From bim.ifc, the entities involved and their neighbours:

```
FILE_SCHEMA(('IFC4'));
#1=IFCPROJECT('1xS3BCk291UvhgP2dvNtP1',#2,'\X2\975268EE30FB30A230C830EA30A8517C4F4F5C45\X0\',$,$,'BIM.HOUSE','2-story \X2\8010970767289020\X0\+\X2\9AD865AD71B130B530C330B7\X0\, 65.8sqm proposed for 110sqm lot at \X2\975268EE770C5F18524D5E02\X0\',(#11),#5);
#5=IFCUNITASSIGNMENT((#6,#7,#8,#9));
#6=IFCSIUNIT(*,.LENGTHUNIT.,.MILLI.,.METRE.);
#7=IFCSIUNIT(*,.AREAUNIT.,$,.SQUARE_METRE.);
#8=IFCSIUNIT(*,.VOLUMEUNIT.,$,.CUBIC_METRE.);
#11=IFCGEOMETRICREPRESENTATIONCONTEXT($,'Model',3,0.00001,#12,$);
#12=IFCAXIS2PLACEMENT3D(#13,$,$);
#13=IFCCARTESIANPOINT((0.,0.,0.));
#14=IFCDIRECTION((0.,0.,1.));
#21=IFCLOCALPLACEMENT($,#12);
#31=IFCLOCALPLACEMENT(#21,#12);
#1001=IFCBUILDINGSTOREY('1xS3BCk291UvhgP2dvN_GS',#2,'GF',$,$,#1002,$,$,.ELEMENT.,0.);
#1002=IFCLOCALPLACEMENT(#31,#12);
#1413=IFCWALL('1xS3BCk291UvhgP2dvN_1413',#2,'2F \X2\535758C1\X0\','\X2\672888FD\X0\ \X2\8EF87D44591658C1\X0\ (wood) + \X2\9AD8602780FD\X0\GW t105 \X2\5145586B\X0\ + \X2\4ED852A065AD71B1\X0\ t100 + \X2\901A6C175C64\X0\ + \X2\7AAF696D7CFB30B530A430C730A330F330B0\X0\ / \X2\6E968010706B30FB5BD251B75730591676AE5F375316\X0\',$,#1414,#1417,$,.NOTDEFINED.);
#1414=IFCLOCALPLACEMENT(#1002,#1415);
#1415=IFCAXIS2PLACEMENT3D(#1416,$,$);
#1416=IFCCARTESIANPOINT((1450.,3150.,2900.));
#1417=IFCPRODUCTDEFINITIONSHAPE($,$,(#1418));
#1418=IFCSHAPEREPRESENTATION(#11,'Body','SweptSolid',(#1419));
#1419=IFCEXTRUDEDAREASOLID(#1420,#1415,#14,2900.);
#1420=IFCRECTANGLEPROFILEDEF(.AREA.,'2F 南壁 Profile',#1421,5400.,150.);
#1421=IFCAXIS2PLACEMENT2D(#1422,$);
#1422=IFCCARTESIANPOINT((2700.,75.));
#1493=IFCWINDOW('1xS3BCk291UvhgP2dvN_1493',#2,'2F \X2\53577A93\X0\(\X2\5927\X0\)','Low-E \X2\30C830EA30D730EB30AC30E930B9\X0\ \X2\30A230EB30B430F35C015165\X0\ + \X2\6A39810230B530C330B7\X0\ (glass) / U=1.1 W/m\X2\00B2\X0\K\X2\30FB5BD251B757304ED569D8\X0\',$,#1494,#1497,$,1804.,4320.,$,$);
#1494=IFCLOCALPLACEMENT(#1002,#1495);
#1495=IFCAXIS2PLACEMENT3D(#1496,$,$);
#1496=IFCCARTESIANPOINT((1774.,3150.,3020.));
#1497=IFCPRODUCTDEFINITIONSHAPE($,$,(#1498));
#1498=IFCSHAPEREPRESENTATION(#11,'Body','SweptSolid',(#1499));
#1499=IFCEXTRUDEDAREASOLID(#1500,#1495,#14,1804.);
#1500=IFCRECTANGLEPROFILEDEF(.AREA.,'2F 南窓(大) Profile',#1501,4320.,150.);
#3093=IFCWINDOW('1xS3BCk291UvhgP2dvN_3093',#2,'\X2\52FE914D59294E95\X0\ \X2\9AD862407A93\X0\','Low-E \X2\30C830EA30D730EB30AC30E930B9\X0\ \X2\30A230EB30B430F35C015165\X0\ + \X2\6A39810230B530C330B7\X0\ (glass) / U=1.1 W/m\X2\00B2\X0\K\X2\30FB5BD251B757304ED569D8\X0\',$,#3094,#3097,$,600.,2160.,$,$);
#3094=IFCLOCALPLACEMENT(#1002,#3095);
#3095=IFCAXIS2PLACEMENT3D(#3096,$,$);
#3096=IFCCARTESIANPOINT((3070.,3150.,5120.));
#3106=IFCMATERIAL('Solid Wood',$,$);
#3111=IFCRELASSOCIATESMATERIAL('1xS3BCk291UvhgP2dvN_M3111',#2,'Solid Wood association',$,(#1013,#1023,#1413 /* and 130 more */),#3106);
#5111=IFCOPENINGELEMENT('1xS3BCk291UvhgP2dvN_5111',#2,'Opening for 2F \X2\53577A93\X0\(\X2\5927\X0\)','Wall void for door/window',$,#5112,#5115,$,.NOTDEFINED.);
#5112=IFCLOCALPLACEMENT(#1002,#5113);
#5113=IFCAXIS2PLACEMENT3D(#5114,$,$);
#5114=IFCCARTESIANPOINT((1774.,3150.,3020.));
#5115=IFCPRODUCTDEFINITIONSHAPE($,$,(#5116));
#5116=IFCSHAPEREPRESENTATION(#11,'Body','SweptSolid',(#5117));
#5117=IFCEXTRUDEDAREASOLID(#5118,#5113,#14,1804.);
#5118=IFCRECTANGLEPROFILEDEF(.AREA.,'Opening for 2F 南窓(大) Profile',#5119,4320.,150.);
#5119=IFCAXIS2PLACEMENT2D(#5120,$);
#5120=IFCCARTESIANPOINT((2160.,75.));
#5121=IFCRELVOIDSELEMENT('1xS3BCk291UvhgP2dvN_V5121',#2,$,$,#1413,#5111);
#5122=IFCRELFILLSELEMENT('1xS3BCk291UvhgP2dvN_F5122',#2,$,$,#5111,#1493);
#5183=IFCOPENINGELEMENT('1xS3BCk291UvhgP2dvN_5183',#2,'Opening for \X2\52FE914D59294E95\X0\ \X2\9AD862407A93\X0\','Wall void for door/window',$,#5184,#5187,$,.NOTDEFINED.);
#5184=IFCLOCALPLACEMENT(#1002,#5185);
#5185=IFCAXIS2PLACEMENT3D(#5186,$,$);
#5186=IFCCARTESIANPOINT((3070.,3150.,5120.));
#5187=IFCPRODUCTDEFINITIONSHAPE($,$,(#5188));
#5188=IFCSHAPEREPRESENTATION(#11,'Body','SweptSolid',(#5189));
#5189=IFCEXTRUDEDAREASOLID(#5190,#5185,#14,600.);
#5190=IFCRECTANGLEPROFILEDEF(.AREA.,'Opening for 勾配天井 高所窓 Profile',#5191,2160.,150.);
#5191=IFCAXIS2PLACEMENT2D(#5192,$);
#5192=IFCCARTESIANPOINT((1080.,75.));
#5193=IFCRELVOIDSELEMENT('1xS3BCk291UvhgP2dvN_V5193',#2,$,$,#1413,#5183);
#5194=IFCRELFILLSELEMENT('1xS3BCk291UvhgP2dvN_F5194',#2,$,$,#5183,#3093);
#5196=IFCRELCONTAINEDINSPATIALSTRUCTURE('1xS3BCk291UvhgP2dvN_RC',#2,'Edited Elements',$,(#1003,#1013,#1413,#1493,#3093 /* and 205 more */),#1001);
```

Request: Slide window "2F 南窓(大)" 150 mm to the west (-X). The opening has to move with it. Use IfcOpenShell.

```python
import ifcopenshell
import ifcopenshell.api.geometry
import ifcopenshell.util.placement

model = ifcopenshell.open("bim.ifc")

window = model.by_id(1493)
opening = window.FillsVoids[0].RelatingOpeningElement
wall = opening.VoidsElements[0].RelatingBuildingElement

wall_matrix = ifcopenshell.util.placement.get_local_placement(wall.ObjectPlacement)
shift = wall_matrix[:3, 0] * -150.0
before = ifcopenshell.util.placement.get_local_placement(window.ObjectPlacement)[:3, 3].copy()

# The window is not placed relative to its opening, so move both.
for product in (opening, window):
    matrix = ifcopenshell.util.placement.get_local_placement(product.ObjectPlacement)
    matrix[:3, 3] += shift
    ifcopenshell.api.geometry.edit_object_placement(model, product=product, matrix=matrix, is_si=False)

after = ifcopenshell.util.placement.get_local_placement(window.ObjectPlacement)[:3, 3]
print("window moved by", (after - before).round(3) + 0.0)

model.write("bim_edited.ifc")
```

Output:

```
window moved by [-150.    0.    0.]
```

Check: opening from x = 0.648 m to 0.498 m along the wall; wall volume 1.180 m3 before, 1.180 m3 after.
